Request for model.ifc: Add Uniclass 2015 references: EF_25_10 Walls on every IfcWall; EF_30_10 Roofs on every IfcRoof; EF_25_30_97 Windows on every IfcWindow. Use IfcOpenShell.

First a look at what the model holds.

```python
import ifcopenshell

model = ifcopenshell.open("model.ifc")
print(model.schema)
print("classifications:", [c.Name for c in model.by_type("IfcClassification")])
for ifc_class in ("IfcDoor", "IfcRoof", "IfcStair", "IfcWall", "IfcWindow"):
    print(ifc_class, len(model.by_type(ifc_class)))
```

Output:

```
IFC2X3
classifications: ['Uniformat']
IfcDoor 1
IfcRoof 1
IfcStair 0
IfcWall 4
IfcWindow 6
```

```python
import ifcopenshell
import ifcopenshell.api.classification

model = ifcopenshell.open("model.ifc")

# IFC2X3 requires Source and Edition and has no link from the project to the system.
system = model.create_entity("IfcClassification", Source="NBS", Edition="2015", Name="Uniclass 2015")

codes = {
    "IfcWall": ("EF_25_10", "Walls"),
    "IfcRoof": ("EF_30_10", "Roofs"),
    "IfcWindow": ("EF_25_30_97", "Windows"),
}
for ifc_class, (code, name) in codes.items():
    products = model.by_type(ifc_class)
    ifcopenshell.api.classification.add_reference(
        model, products=products, classification=system, identification=code, name=name
    )
    print(code, len(products))

model.write("model_v2.ifc")
```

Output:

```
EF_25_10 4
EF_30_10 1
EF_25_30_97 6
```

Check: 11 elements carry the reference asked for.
